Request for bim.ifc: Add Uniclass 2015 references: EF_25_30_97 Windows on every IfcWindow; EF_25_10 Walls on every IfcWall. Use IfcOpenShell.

First a look at what the model holds.

```python
import ifcopenshell

model = ifcopenshell.open("bim.ifc")
print(model.schema)
print("classifications:", [c.Name for c in model.by_type("IfcClassification")])
for ifc_class in ("IfcDoor", "IfcRoof", "IfcStair", "IfcWall", "IfcWindow"):
    print(ifc_class, len(model.by_type(ifc_class)))
```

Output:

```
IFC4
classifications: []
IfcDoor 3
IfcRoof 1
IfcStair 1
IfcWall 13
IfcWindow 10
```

```python
import ifcopenshell
import ifcopenshell.api.classification

model = ifcopenshell.open("bim.ifc")

system = ifcopenshell.api.classification.add_classification(model, classification="Uniclass 2015")

codes = {
    "IfcWindow": ("EF_25_30_97", "Windows"),
    "IfcWall": ("EF_25_10", "Walls"),
}
for ifc_class, (code, name) in codes.items():
    products = model.by_type(ifc_class)
    ifcopenshell.api.classification.add_reference(
        model, products=products, classification=system, identification=code, name=name
    )
    print(code, len(products))

model.write("bim-out.ifc")
```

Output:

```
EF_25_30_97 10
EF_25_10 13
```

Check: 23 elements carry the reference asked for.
